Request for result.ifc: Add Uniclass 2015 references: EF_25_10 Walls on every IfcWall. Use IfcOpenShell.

First a look at what the model holds.

```python
import ifcopenshell

model = ifcopenshell.open("result.ifc")
print(model.schema)
print("classifications:", [c.Name for c in model.by_type("IfcClassification")])
for ifc_class in ("IfcDoor", "IfcRoof", "IfcStair", "IfcWall", "IfcWindow"):
    print(ifc_class, len(model.by_type(ifc_class)))
```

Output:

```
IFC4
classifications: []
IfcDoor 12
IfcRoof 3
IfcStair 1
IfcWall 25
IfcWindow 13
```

```python
import ifcopenshell
import ifcopenshell.api.classification

model = ifcopenshell.open("result.ifc")

system = ifcopenshell.api.classification.add_classification(model, classification="Uniclass 2015")

codes = {
    "IfcWall": ("EF_25_10", "Walls"),
}
for ifc_class, (code, name) in codes.items():
    products = model.by_type(ifc_class)
    ifcopenshell.api.classification.add_reference(
        model, products=products, classification=system, identification=code, name=name
    )
    print(code, len(products))

model.write("result_edited.ifc")
```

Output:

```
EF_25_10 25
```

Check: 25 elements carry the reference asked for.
